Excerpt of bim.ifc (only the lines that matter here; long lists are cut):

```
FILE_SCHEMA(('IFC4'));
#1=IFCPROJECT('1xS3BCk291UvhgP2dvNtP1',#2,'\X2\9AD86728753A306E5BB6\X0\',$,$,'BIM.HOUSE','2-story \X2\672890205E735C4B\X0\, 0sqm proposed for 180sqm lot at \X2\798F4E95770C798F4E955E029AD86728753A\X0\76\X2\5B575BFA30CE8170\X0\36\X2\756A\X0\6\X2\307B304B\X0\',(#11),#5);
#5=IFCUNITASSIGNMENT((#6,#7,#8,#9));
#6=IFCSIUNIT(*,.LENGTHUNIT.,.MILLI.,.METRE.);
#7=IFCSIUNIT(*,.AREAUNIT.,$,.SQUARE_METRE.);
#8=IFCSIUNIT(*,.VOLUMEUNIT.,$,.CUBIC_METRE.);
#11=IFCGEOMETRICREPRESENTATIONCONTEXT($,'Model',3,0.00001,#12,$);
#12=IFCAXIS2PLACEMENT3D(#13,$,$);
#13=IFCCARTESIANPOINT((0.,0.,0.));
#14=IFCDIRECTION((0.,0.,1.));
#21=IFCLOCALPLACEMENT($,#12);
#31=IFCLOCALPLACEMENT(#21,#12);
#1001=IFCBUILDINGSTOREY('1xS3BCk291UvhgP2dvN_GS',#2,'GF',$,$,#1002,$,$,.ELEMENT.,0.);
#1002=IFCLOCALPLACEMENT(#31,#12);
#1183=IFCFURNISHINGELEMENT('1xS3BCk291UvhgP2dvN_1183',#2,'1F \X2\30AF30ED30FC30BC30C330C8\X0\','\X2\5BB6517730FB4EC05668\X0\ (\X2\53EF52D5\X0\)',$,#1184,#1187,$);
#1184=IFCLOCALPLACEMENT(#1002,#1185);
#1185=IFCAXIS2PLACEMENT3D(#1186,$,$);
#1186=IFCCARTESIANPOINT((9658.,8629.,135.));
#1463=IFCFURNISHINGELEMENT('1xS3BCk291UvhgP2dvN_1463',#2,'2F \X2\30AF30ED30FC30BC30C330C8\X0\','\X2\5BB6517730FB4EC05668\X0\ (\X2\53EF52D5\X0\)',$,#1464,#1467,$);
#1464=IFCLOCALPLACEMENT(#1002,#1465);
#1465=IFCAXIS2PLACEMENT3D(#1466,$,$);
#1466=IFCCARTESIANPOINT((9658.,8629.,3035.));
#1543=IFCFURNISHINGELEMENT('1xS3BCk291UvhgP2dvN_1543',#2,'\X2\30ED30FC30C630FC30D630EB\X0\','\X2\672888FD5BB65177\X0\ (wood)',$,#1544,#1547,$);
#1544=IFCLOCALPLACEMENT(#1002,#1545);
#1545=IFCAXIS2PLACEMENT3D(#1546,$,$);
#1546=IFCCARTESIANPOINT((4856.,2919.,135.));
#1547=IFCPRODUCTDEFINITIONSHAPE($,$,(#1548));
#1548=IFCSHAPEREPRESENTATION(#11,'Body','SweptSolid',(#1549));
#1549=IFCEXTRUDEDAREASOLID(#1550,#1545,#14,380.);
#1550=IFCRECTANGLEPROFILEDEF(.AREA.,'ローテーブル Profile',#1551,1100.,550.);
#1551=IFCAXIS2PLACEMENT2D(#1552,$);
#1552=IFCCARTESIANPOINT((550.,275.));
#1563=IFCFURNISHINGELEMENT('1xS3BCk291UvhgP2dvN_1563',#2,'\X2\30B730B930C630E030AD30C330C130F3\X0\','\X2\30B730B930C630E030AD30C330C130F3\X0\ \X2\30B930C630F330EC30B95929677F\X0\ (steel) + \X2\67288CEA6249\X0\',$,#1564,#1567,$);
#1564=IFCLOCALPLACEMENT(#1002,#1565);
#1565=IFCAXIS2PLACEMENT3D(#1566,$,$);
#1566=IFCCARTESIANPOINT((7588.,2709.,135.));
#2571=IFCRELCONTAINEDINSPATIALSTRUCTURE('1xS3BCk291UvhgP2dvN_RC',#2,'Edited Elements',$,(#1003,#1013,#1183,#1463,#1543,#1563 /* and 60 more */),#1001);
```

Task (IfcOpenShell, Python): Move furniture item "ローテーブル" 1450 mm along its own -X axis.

```python
import ifcopenshell
import ifcopenshell.api.geometry
import ifcopenshell.util.placement

model = ifcopenshell.open("bim.ifc")

item = model.by_guid("1xS3BCk291UvhgP2dvN_1543")
matrix = ifcopenshell.util.placement.get_local_placement(item.ObjectPlacement)
matrix[:3, 3] -= matrix[:3, 0] * 1450.0
ifcopenshell.api.geometry.edit_object_placement(model, product=item, matrix=matrix, is_si=False)

print(ifcopenshell.util.placement.get_local_placement(item.ObjectPlacement).round(3) + 0.0)

model.write("bim_edited.ifc")
```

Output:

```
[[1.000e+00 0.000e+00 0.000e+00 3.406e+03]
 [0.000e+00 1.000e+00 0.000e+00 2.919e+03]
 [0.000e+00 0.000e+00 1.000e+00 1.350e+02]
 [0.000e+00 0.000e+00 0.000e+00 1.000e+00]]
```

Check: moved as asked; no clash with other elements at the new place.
